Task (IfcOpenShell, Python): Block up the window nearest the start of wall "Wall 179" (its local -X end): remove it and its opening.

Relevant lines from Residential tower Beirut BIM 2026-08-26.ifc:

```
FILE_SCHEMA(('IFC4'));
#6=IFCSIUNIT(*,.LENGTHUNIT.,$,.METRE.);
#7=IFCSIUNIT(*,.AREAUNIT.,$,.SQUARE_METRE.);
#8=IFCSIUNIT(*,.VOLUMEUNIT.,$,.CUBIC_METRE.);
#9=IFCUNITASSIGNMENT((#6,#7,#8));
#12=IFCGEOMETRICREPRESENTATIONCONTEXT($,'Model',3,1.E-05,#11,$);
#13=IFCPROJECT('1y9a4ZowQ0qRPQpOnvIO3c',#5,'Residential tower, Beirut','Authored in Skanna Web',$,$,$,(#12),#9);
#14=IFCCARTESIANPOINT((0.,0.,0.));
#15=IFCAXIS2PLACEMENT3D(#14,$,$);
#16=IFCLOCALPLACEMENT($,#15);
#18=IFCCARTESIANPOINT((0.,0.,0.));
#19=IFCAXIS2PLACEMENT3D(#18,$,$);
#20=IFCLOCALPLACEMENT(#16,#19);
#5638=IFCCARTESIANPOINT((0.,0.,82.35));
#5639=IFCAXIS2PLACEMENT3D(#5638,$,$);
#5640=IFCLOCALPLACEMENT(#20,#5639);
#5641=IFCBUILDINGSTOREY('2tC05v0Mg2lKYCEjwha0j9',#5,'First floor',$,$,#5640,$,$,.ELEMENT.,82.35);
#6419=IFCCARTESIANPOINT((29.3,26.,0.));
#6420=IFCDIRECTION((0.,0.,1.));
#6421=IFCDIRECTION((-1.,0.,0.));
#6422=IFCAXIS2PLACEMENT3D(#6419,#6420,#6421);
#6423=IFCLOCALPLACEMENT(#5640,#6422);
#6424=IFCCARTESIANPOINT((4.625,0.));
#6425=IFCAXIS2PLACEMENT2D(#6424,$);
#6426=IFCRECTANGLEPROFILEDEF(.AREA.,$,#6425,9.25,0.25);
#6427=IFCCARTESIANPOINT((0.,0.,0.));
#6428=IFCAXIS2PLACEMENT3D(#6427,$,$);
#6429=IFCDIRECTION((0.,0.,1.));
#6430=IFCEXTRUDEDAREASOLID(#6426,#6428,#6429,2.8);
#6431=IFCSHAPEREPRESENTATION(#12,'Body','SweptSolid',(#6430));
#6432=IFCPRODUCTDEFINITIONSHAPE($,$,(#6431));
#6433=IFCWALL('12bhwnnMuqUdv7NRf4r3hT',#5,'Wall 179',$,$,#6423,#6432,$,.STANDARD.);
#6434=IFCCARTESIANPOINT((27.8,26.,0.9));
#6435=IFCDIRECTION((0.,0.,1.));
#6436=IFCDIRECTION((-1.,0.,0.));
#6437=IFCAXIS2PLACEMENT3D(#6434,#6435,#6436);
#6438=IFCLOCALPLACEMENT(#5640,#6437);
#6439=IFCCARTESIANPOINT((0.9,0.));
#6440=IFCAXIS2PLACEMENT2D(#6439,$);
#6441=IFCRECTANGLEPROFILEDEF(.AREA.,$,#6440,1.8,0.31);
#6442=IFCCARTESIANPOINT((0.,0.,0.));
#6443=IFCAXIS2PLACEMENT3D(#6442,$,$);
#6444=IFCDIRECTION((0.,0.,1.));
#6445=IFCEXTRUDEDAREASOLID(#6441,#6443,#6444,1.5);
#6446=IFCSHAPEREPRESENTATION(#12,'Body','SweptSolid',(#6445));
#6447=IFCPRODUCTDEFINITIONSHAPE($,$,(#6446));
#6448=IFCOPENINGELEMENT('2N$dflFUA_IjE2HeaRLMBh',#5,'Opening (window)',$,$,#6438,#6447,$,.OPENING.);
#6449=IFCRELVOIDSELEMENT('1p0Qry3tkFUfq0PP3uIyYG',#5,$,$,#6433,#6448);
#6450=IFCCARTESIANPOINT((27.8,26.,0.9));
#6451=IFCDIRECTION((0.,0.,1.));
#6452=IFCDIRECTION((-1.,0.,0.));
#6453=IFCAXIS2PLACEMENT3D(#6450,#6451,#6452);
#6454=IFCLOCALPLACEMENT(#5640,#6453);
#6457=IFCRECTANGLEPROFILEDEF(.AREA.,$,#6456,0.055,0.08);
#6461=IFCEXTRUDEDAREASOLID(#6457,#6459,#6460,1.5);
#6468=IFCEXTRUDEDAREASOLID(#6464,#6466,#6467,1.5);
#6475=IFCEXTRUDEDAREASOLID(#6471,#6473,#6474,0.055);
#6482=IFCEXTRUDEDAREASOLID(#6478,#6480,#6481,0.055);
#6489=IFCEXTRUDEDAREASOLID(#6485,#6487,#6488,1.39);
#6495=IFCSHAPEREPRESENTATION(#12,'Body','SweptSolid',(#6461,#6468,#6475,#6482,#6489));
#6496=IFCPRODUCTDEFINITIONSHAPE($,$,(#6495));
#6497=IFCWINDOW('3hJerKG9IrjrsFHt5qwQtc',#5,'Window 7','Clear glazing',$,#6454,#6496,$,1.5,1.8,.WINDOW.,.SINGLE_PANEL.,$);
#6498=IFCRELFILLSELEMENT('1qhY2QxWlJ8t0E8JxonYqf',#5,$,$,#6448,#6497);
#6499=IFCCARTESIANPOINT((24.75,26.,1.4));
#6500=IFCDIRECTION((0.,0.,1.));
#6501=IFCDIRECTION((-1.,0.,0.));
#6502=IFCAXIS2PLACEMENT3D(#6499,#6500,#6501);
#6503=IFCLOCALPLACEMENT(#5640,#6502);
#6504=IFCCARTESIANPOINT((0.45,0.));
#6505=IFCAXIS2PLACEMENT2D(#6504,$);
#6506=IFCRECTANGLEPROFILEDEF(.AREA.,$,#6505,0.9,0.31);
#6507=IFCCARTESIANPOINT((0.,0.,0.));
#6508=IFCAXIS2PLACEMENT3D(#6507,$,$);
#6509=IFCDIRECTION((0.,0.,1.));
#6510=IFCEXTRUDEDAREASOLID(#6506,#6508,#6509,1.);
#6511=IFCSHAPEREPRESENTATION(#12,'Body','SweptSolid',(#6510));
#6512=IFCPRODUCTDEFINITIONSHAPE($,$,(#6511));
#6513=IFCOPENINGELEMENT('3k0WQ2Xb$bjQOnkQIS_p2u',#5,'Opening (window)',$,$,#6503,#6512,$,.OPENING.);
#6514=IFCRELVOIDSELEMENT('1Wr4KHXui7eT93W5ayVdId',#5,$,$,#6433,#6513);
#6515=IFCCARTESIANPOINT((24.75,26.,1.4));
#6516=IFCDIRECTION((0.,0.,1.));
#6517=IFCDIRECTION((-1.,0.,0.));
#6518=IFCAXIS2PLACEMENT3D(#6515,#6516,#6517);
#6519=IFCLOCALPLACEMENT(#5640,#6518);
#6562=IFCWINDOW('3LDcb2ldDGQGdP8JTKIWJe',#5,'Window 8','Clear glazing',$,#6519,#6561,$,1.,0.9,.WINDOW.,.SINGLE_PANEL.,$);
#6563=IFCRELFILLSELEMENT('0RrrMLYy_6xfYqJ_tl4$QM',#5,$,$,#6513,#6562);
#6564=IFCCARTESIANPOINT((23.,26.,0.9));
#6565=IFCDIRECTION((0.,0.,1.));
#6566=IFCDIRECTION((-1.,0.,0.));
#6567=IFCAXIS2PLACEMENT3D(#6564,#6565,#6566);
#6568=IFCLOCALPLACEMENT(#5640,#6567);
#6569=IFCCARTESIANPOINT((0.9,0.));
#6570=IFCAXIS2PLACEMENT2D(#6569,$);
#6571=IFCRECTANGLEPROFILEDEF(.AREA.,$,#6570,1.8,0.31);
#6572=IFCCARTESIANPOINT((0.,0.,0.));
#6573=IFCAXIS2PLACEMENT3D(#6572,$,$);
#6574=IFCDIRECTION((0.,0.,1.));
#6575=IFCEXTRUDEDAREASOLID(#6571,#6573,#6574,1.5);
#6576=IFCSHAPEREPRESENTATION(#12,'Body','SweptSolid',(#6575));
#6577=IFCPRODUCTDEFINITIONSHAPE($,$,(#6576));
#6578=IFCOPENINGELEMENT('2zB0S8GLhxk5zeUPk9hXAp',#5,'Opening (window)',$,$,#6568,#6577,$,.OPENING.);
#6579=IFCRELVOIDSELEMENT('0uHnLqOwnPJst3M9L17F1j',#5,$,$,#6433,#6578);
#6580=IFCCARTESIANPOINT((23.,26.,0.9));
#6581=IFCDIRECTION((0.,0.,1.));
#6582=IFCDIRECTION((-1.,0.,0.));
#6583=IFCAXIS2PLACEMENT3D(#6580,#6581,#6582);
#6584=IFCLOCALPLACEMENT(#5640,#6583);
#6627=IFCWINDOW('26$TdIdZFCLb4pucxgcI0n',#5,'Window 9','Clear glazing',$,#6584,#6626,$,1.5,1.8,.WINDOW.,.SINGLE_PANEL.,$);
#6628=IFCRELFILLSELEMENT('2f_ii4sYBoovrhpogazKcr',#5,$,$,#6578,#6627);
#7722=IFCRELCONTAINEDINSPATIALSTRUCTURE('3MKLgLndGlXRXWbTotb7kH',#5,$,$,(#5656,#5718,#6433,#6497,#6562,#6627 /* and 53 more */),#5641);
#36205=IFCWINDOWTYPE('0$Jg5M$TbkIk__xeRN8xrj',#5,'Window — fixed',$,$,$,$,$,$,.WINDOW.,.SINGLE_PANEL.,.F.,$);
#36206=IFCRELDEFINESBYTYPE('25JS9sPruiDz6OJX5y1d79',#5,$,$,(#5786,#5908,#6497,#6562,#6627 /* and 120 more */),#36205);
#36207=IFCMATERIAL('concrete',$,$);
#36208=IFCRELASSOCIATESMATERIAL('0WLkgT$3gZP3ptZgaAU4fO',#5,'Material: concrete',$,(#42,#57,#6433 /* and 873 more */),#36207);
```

```python
import ifcopenshell
import ifcopenshell.api.feature
import ifcopenshell.api.root
import ifcopenshell.geom
import ifcopenshell.util.shape

model = ifcopenshell.open("Residential tower Beirut BIM 2026-08-26.ifc")
settings = ifcopenshell.geom.settings()


def volume(element):
    """Net volume in cubic metres, openings subtracted."""
    shape = ifcopenshell.geom.create_shape(settings, element)
    return ifcopenshell.util.shape.get_volume(shape.geometry)


window = model.by_guid("3hJerKG9IrjrsFHt5qwQtc")
opening = window.FillsVoids[0].RelatingOpeningElement
wall = opening.VoidsElements[0].RelatingBuildingElement
before = volume(wall)

ifcopenshell.api.root.remove_product(model, product=window)
ifcopenshell.api.feature.remove_feature(model, feature=opening)

after = volume(wall)

print(f"wall volume {before:.3f} -> {after:.3f} m3")

model.write("Residential tower Beirut BIM 2026-08-26_rev.ifc")
```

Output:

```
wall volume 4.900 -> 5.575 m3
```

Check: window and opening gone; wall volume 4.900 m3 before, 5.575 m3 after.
